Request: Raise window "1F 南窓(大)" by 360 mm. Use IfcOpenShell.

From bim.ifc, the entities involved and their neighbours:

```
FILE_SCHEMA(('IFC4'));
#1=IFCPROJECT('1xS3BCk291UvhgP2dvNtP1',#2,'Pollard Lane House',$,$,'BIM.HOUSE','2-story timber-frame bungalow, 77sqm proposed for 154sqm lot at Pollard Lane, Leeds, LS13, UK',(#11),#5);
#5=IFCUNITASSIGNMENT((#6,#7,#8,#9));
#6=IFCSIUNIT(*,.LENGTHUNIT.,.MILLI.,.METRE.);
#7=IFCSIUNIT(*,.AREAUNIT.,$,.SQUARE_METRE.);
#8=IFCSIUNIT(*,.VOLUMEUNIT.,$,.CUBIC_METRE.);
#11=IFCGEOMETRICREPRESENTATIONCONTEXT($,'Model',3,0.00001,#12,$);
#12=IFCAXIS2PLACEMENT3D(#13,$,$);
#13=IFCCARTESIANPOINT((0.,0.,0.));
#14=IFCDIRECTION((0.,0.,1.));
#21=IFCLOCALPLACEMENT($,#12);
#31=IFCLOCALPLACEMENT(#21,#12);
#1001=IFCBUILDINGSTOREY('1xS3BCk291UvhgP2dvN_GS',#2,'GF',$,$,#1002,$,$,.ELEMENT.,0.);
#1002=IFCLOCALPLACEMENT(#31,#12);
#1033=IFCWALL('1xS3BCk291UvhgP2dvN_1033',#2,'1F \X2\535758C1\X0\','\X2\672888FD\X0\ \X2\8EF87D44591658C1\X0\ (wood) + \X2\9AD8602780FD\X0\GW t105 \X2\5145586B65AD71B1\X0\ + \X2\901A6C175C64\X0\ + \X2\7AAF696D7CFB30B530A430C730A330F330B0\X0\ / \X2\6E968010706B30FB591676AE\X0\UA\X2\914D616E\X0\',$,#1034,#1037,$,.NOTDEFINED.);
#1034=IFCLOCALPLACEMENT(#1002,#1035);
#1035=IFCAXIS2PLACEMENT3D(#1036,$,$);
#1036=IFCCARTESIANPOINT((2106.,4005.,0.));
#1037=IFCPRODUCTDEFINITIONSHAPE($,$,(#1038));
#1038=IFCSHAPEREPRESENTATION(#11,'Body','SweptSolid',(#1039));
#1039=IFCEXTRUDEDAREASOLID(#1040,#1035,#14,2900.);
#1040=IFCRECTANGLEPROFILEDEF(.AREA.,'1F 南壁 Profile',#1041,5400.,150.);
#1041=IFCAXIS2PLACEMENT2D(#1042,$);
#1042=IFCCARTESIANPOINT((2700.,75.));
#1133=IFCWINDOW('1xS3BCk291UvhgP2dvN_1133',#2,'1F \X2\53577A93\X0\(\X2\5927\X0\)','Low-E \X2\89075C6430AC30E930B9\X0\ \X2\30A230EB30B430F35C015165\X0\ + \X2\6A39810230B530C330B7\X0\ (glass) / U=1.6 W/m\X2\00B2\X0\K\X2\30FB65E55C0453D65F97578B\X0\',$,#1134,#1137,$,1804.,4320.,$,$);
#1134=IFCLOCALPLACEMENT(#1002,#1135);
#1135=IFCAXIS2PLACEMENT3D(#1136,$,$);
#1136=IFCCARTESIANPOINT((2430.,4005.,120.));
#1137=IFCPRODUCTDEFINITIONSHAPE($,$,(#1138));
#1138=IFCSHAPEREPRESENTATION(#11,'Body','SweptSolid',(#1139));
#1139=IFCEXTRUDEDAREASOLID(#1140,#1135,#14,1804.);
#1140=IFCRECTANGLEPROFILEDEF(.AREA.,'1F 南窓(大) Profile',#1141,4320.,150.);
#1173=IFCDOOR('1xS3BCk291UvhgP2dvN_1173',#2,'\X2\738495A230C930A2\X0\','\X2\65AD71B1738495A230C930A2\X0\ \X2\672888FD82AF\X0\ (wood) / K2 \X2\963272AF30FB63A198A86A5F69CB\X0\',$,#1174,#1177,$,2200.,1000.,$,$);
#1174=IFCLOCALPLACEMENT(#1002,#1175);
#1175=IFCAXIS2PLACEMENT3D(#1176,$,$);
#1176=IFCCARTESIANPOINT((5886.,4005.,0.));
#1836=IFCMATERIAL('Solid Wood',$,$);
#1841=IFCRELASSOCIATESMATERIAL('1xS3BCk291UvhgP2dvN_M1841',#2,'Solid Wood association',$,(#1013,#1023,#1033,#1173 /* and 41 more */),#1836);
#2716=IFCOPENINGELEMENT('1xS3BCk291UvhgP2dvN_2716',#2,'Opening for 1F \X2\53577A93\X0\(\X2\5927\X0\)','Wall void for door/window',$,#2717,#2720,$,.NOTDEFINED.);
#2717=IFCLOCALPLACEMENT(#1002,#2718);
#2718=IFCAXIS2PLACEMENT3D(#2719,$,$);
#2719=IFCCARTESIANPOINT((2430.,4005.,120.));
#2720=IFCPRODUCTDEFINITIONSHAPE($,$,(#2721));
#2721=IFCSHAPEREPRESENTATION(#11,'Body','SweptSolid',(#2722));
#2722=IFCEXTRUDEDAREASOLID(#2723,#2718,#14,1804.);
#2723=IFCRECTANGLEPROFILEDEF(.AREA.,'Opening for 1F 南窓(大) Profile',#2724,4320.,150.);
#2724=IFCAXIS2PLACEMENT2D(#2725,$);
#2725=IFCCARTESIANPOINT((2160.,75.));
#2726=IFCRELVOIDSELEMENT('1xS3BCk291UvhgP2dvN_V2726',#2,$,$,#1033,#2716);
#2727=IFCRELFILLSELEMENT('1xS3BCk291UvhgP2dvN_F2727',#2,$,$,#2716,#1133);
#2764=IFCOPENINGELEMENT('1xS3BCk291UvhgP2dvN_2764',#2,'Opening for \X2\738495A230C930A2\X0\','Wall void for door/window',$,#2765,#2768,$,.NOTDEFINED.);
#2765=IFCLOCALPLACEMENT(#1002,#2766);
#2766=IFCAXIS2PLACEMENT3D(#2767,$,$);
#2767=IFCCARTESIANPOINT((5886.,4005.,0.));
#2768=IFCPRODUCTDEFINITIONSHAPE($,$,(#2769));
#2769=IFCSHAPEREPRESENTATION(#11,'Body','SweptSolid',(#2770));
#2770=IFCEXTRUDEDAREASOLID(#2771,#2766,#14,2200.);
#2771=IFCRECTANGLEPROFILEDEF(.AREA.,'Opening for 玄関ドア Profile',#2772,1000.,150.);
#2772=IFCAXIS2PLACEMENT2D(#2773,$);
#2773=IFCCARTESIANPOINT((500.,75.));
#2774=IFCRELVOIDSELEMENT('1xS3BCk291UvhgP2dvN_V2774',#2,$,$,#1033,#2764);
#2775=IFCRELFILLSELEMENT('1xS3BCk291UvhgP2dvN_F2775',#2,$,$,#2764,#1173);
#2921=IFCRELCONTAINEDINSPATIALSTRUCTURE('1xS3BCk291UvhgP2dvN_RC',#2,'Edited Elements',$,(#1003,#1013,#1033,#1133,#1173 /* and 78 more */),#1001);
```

```python
import numpy as np
import ifcopenshell
import ifcopenshell.api.geometry
import ifcopenshell.util.placement
import ifcopenshell.util.unit

model = ifcopenshell.open("bim.ifc")
unit_scale = ifcopenshell.util.unit.calculate_unit_scale(model)

window = model.by_guid("1xS3BCk291UvhgP2dvN_1133")
opening = window.FillsVoids[0].RelatingOpeningElement
dz = 360.0

shift = np.array([0.0, 0.0, dz])
# The window is not placed relative to its opening, so move both.
for product in (opening, window):
    matrix = ifcopenshell.util.placement.get_local_placement(product.ObjectPlacement)
    matrix[:3, 3] += shift
    ifcopenshell.api.geometry.edit_object_placement(model, product=product, matrix=matrix, is_si=False)

print(f"moved by {dz * unit_scale:+.3f} m")

model.write("bim_v2.ifc")
```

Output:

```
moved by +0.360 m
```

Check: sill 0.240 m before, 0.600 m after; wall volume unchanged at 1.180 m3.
